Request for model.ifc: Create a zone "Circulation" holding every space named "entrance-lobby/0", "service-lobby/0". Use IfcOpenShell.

First a look at what the model holds.

```python
import ifcopenshell

model = ifcopenshell.open("model.ifc")
print(model.schema)
seen = {}
for space in model.by_type("IfcSpace"):
    seen[space.Name] = seen.get(space.Name, 0) + 1
for name, count in sorted(seen.items(), key=str):
    print(count, "x", name)
print("zones:", [z.Name for z in model.by_type("IfcZone")][:20])
```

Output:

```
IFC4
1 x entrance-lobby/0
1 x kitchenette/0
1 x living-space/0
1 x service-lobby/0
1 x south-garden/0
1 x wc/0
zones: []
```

```python
import ifcopenshell
import ifcopenshell.api.group
import ifcopenshell.api.root

model = ifcopenshell.open("model.ifc")

names = {"entrance-lobby/0", "service-lobby/0"}
spaces = [s for s in model.by_type("IfcSpace") if s.Name in names]

zone = ifcopenshell.api.root.create_entity(model, ifc_class="IfcZone", name="Circulation")
ifcopenshell.api.group.assign_group(model, products=spaces, group=zone)
print(len(spaces), "spaces in", zone.Name)

model.write("model_edited.ifc")
```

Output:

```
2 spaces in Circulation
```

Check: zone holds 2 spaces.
